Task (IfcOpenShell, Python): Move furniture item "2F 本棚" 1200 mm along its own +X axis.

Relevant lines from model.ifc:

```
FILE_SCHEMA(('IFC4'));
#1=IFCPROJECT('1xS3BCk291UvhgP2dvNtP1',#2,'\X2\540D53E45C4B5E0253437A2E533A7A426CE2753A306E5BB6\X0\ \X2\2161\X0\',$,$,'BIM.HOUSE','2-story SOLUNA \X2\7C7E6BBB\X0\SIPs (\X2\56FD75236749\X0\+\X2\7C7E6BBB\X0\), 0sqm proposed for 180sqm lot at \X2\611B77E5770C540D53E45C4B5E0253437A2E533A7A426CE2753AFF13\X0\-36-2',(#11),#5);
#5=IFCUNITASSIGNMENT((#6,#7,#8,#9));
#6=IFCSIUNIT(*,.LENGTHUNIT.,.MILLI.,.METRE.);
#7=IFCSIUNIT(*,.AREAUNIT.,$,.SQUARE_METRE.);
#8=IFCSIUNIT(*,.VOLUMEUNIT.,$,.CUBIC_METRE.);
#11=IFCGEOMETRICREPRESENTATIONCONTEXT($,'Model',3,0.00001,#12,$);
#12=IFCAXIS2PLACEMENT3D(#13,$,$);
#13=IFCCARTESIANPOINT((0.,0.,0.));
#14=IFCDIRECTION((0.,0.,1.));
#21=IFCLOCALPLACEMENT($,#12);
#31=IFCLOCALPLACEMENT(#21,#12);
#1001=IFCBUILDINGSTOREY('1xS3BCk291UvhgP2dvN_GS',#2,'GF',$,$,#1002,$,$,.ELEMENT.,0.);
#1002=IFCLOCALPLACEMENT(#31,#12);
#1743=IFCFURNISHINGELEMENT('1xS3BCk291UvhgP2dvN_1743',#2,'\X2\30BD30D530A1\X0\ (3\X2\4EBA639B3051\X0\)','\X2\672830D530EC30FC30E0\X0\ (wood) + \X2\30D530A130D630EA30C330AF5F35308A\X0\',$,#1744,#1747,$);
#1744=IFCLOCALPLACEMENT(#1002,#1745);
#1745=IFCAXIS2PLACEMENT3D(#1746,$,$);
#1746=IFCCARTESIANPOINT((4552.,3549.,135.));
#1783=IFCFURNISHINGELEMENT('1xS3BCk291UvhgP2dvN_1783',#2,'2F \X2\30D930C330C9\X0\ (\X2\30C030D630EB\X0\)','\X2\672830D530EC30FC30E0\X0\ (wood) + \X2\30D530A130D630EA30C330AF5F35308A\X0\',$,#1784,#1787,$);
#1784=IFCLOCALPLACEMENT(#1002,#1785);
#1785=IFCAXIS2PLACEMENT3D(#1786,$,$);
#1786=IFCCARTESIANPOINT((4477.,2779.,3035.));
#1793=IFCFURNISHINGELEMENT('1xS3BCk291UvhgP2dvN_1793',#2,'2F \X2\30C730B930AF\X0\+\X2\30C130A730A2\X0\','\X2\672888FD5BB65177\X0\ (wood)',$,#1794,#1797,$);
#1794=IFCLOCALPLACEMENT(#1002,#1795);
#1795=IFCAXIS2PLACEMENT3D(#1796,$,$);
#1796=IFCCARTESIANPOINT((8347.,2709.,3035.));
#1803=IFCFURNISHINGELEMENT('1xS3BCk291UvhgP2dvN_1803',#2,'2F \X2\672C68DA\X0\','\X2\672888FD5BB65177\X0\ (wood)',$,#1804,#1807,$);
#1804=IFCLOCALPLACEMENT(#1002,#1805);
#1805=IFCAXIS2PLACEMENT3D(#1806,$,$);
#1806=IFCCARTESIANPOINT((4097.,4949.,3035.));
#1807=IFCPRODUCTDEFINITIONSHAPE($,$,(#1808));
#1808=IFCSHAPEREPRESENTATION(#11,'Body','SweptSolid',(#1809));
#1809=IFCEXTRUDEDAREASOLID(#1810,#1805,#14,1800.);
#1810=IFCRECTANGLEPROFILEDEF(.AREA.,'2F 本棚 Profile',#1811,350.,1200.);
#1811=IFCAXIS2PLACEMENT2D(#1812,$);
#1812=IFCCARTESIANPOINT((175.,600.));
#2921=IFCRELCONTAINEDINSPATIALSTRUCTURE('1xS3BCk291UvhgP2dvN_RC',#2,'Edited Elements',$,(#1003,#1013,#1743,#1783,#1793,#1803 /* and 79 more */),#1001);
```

```python
import ifcopenshell
import ifcopenshell.api.geometry
import ifcopenshell.util.placement
import ifcopenshell.util.unit

model = ifcopenshell.open("model.ifc")
unit_scale = ifcopenshell.util.unit.calculate_unit_scale(model)

item = model.by_guid("1xS3BCk291UvhgP2dvN_1803")
matrix = ifcopenshell.util.placement.get_local_placement(item.ObjectPlacement)
matrix[:3, 3] += matrix[:3, 0] * 1.2 / unit_scale
ifcopenshell.api.geometry.edit_object_placement(model, product=item, matrix=matrix, is_si=False)

print(ifcopenshell.util.placement.get_local_placement(item.ObjectPlacement).round(3) + 0.0)

model.write("model_v2.ifc")
```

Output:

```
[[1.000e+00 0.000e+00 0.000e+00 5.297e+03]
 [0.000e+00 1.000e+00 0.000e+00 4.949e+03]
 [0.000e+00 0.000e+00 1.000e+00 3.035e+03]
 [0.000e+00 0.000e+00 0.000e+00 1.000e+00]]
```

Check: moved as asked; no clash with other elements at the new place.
